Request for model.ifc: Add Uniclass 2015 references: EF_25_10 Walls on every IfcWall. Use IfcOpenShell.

First a look at what the model holds.

```python
import ifcopenshell

model = ifcopenshell.open("model.ifc")
print(model.schema)
print("classifications:", [c.Name for c in model.by_type("IfcClassification")])
for ifc_class in ("IfcDoor", "IfcRoof", "IfcStair", "IfcWall", "IfcWindow"):
    print(ifc_class, len(model.by_type(ifc_class)))
```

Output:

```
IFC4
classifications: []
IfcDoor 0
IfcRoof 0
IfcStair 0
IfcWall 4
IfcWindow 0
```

```python
import ifcopenshell
import ifcopenshell.api.classification

model = ifcopenshell.open("model.ifc")

system = ifcopenshell.api.classification.add_classification(model, classification="Uniclass 2015")

codes = {
    "IfcWall": ("EF_25_10", "Walls"),
}
for ifc_class, (code, name) in codes.items():
    products = model.by_type(ifc_class)
    ifcopenshell.api.classification.add_reference(
        model, products=products, classification=system, identification=code, name=name
    )
    print(code, len(products))

model.write("model_v2.ifc")
```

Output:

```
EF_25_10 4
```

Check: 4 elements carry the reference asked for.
